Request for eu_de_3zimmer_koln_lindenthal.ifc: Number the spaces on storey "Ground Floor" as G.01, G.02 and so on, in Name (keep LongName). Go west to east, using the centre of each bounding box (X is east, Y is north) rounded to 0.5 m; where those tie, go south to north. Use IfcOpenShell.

First a look at what the model holds.

```python
import ifcopenshell
import ifcopenshell.util.element
import ifcopenshell.util.placement

model = ifcopenshell.open("eu_de_3zimmer_koln_lindenthal.ifc")
print(model.schema)
storey = next(s for s in model.by_type("IfcBuildingStorey") if s.Name == "Ground Floor")
spaces = [e for e in ifcopenshell.util.element.get_decomposition(storey) if e.is_a("IfcSpace")]
for e in sorted(spaces, key=lambda e: e.id()):
    origin = ifcopenshell.util.placement.get_local_placement(e.ObjectPlacement)[:3, 3]
    print(e.id(), e.Name, e.LongName, origin.round(2) + 0.0, sep=" | ")
```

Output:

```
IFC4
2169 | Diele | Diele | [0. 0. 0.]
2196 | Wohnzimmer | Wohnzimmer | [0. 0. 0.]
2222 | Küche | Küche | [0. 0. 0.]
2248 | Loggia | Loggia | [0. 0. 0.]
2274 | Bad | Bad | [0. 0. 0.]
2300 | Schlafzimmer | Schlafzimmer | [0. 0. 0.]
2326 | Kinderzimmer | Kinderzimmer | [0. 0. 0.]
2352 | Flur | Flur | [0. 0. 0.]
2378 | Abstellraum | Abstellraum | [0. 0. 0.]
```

```python
import ifcopenshell
import ifcopenshell.geom
import ifcopenshell.util.element
import ifcopenshell.util.shape

model = ifcopenshell.open("eu_de_3zimmer_koln_lindenthal.ifc")
settings = ifcopenshell.geom.settings()
settings.set("use-world-coords", True)


def centre(element):
    shape = ifcopenshell.geom.create_shape(settings, element)
    return ifcopenshell.util.shape.get_bbox_centroid(shape.geometry)


storey = next(s for s in model.by_type("IfcBuildingStorey") if s.Name == "Ground Floor")
spaces = [e for e in ifcopenshell.util.element.get_decomposition(storey) if e.is_a("IfcSpace")]

# Insertion points can sit at a corner or the storey origin, so sort by the geometry (in metres).
centres = {e: centre(e) for e in spaces}
spaces.sort(key=lambda e: (round(centres[e][0] / 0.5), centres[e][1]))

for i, e in enumerate(spaces, start=1):
    number = f"G.{i:02d}"
    e.Name = number
    print(e.id(), number)

model.write("eu_de_3zimmer_koln_lindenthal_v2.ifc")
```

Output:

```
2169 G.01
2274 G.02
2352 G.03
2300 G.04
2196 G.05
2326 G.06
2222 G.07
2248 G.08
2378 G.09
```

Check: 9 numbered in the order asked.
